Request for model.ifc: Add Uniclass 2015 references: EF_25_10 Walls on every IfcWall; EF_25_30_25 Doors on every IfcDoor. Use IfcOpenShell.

First a look at what the model holds.

```python
import ifcopenshell

model = ifcopenshell.open("model.ifc")
print(model.schema)
print("classifications:", [c.Name for c in model.by_type("IfcClassification")])
for ifc_class in ("IfcDoor", "IfcRoof", "IfcStair", "IfcWall", "IfcWindow"):
    print(ifc_class, len(model.by_type(ifc_class)))
```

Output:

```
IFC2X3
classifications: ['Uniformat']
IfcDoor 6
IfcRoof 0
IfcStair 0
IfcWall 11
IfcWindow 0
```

```python
import ifcopenshell
import ifcopenshell.api.classification

model = ifcopenshell.open("model.ifc")

# IFC2X3 requires Source and Edition and has no link from the project to the system.
system = model.create_entity("IfcClassification", Source="NBS", Edition="2015", Name="Uniclass 2015")

codes = {
    "IfcWall": ("EF_25_10", "Walls"),
    "IfcDoor": ("EF_25_30_25", "Doors"),
}
for ifc_class, (code, name) in codes.items():
    products = model.by_type(ifc_class)
    ifcopenshell.api.classification.add_reference(
        model, products=products, classification=system, identification=code, name=name
    )
    print(code, len(products))

model.write("model_updated.ifc")
```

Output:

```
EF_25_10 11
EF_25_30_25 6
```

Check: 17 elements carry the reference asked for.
